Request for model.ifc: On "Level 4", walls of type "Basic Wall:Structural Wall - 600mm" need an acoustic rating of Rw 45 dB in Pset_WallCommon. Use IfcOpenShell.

First a look at what the model holds.

```python
import ifcopenshell
import ifcopenshell.util.element

model = ifcopenshell.open("model.ifc")
print(model.schema)
storey = next(s for s in model.by_type("IfcBuildingStorey") if s.Name == "Level 4")
walls = [e for e in ifcopenshell.util.element.get_decomposition(storey) if e.is_a("IfcWall")]
seen = {}
for e in walls:
    element_type = ifcopenshell.util.element.get_type(e)
    key = (element_type.Name if element_type != e and element_type else None, ifcopenshell.util.element.get_pset(e, "Pset_WallCommon", "AcousticRating"))
    seen[key] = seen.get(key, 0) + 1
for (name, value), count in sorted(seen.items(), key=str):
    print(count, "x", name, "|", value)
```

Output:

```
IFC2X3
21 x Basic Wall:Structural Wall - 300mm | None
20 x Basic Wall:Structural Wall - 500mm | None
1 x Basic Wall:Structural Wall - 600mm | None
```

```python
import ifcopenshell
import ifcopenshell.api.pset
import ifcopenshell.util.element

model = ifcopenshell.open("model.ifc")

storey = next(s for s in model.by_type("IfcBuildingStorey") if s.Name == "Level 4")
walls = [e for e in ifcopenshell.util.element.get_decomposition(storey) if e.is_a("IfcWall")]

count = 0
for e in walls:
    element_type = ifcopenshell.util.element.get_type(e)
    if element_type in (None, e) or element_type.Name != "Basic Wall:Structural Wall - 600mm":
        continue
    # add_pset returns the element's existing set when there is one.
    pset = ifcopenshell.api.pset.add_pset(model, product=e, name="Pset_WallCommon")
    ifcopenshell.api.pset.edit_pset(model, pset=pset, properties={"AcousticRating": "Rw 45 dB"})
    count += 1

print(count, "walls updated")

model.write("model-out.ifc")
```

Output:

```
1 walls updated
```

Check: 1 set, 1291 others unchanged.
